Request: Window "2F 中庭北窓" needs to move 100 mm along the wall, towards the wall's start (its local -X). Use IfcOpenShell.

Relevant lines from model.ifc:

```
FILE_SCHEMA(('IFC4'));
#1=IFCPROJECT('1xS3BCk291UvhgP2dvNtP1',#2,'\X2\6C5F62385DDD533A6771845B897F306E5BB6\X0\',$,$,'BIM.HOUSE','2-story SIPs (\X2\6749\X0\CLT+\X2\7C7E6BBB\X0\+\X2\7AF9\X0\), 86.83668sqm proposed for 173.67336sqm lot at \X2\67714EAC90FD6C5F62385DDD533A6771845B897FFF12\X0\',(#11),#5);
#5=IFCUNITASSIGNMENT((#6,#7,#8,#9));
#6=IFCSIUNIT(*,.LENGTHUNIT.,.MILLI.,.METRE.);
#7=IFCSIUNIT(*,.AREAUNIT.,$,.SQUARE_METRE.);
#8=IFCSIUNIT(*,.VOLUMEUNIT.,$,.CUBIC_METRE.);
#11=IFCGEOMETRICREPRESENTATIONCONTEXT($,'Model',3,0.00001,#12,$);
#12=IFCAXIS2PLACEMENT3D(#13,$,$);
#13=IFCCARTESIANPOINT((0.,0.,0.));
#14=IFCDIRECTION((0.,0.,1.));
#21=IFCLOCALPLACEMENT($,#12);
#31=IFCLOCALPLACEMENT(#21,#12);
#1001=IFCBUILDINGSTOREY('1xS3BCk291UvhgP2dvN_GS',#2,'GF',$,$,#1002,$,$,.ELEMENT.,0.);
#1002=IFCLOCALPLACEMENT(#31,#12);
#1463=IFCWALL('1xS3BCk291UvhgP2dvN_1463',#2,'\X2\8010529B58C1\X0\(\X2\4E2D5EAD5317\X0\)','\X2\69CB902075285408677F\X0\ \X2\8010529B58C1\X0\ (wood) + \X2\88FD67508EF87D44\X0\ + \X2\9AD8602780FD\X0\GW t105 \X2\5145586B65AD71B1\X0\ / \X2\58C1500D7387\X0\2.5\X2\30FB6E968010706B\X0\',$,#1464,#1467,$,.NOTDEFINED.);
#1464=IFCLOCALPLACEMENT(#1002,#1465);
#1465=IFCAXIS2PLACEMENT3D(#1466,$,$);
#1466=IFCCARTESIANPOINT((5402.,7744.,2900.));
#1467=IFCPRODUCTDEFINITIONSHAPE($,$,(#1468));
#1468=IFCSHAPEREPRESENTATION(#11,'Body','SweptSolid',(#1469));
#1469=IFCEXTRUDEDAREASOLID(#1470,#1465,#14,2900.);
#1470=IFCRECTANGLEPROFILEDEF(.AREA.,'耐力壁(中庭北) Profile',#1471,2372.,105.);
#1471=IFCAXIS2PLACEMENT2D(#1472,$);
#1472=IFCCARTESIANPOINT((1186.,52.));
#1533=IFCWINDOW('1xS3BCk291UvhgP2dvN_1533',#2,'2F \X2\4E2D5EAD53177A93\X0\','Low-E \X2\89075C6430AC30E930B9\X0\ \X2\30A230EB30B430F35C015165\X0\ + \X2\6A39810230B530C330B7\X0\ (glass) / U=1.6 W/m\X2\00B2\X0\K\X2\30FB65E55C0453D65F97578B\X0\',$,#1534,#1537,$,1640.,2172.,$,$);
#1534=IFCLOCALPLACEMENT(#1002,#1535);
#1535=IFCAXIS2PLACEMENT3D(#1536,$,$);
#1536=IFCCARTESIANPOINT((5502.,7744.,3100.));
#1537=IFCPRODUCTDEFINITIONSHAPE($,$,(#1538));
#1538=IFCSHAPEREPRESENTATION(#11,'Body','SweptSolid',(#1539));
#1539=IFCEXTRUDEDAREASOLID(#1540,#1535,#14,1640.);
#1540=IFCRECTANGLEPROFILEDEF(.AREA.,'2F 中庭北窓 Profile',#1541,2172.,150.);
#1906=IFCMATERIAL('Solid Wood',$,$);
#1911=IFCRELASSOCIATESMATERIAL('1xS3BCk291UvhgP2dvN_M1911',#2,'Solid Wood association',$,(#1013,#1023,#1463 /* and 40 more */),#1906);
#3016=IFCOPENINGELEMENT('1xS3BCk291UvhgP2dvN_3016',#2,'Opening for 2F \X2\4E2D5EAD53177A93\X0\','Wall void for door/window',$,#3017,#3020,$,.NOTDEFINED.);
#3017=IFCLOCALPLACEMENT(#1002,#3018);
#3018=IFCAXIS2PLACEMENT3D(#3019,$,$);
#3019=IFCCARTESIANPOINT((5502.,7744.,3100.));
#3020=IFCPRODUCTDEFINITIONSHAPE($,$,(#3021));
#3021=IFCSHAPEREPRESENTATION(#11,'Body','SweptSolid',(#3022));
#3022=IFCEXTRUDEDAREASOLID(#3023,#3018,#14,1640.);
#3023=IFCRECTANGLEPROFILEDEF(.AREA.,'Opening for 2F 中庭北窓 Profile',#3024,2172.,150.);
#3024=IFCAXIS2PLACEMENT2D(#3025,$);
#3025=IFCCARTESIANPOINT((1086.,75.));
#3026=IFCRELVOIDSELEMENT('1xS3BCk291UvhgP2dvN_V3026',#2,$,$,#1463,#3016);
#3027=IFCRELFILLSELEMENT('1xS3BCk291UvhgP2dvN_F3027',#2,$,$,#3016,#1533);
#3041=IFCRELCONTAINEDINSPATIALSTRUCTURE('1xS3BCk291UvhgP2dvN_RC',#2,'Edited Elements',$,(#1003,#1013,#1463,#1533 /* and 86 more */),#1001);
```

```python
import ifcopenshell
import ifcopenshell.api.geometry
import ifcopenshell.util.placement
import ifcopenshell.util.unit

model = ifcopenshell.open("model.ifc")
unit_scale = ifcopenshell.util.unit.calculate_unit_scale(model)

window = model.by_guid("1xS3BCk291UvhgP2dvN_1533")
opening = window.FillsVoids[0].RelatingOpeningElement
wall = opening.VoidsElements[0].RelatingBuildingElement

wall_matrix = ifcopenshell.util.placement.get_local_placement(wall.ObjectPlacement)
shift = wall_matrix[:3, 0] * -0.1 / unit_scale
before = ifcopenshell.util.placement.get_local_placement(window.ObjectPlacement)[:3, 3].copy()

# The window is not placed relative to its opening, so move both.
for product in (opening, window):
    matrix = ifcopenshell.util.placement.get_local_placement(product.ObjectPlacement)
    matrix[:3, 3] += shift
    ifcopenshell.api.geometry.edit_object_placement(model, product=product, matrix=matrix, is_si=False)

after = ifcopenshell.util.placement.get_local_placement(window.ObjectPlacement)[:3, 3]
print("window moved by", (after - before).round(3) + 0.0)

model.write("model_v2.ifc")
```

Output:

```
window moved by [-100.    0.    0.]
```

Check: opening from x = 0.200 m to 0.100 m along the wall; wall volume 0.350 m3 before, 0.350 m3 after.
